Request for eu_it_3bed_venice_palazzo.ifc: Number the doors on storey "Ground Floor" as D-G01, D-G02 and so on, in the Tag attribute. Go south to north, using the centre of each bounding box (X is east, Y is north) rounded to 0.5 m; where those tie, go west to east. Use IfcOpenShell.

First a look at what the model holds.

```python
import ifcopenshell
import ifcopenshell.util.element
import ifcopenshell.util.placement

model = ifcopenshell.open("eu_it_3bed_venice_palazzo.ifc")
print(model.schema)
storey = next(s for s in model.by_type("IfcBuildingStorey") if s.Name == "Ground Floor")
doors = [e for e in ifcopenshell.util.element.get_decomposition(storey) if e.is_a("IfcDoor")]
for e in sorted(doors, key=lambda e: e.id()):
    origin = ifcopenshell.util.placement.get_local_placement(e.ObjectPlacement)[:3, 3]
    print(e.id(), e.Tag, e.Name, origin.round(2) + 0.0, sep=" | ")
```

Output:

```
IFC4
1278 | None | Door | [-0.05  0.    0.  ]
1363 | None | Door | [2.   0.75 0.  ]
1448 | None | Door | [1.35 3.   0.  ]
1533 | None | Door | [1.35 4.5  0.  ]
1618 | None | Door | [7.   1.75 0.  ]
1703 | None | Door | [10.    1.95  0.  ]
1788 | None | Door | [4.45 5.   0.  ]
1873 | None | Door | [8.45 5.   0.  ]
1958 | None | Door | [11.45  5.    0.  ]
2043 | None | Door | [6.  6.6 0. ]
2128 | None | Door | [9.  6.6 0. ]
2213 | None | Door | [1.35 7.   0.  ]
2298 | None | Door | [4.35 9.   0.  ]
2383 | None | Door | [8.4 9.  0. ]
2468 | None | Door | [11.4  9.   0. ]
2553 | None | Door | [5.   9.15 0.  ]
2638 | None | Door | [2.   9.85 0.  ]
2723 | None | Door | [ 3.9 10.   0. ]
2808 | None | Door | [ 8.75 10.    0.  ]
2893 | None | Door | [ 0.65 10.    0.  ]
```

```python
import ifcopenshell
import ifcopenshell.geom
import ifcopenshell.util.element
import ifcopenshell.util.shape

model = ifcopenshell.open("eu_it_3bed_venice_palazzo.ifc")
settings = ifcopenshell.geom.settings()
settings.set("use-world-coords", True)


def centre(element):
    shape = ifcopenshell.geom.create_shape(settings, element)
    return ifcopenshell.util.shape.get_bbox_centroid(shape.geometry)


storey = next(s for s in model.by_type("IfcBuildingStorey") if s.Name == "Ground Floor")
doors = [e for e in ifcopenshell.util.element.get_decomposition(storey) if e.is_a("IfcDoor")]

# Insertion points can sit at a corner or the storey origin, so sort by the geometry (in metres).
centres = {e: centre(e) for e in doors}
doors.sort(key=lambda e: (round(centres[e][1] / 0.5), centres[e][0]))

for i, e in enumerate(doors, start=1):
    number = f"D-G{i:02d}"
    e.Tag = number
    print(e.id(), number)

model.write("eu_it_3bed_venice_palazzo_updated.ifc")
```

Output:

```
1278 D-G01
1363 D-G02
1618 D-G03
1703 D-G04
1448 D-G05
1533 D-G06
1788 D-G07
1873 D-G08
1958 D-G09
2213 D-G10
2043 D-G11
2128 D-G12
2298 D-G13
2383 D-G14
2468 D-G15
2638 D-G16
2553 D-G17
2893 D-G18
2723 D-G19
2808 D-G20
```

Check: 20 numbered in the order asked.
